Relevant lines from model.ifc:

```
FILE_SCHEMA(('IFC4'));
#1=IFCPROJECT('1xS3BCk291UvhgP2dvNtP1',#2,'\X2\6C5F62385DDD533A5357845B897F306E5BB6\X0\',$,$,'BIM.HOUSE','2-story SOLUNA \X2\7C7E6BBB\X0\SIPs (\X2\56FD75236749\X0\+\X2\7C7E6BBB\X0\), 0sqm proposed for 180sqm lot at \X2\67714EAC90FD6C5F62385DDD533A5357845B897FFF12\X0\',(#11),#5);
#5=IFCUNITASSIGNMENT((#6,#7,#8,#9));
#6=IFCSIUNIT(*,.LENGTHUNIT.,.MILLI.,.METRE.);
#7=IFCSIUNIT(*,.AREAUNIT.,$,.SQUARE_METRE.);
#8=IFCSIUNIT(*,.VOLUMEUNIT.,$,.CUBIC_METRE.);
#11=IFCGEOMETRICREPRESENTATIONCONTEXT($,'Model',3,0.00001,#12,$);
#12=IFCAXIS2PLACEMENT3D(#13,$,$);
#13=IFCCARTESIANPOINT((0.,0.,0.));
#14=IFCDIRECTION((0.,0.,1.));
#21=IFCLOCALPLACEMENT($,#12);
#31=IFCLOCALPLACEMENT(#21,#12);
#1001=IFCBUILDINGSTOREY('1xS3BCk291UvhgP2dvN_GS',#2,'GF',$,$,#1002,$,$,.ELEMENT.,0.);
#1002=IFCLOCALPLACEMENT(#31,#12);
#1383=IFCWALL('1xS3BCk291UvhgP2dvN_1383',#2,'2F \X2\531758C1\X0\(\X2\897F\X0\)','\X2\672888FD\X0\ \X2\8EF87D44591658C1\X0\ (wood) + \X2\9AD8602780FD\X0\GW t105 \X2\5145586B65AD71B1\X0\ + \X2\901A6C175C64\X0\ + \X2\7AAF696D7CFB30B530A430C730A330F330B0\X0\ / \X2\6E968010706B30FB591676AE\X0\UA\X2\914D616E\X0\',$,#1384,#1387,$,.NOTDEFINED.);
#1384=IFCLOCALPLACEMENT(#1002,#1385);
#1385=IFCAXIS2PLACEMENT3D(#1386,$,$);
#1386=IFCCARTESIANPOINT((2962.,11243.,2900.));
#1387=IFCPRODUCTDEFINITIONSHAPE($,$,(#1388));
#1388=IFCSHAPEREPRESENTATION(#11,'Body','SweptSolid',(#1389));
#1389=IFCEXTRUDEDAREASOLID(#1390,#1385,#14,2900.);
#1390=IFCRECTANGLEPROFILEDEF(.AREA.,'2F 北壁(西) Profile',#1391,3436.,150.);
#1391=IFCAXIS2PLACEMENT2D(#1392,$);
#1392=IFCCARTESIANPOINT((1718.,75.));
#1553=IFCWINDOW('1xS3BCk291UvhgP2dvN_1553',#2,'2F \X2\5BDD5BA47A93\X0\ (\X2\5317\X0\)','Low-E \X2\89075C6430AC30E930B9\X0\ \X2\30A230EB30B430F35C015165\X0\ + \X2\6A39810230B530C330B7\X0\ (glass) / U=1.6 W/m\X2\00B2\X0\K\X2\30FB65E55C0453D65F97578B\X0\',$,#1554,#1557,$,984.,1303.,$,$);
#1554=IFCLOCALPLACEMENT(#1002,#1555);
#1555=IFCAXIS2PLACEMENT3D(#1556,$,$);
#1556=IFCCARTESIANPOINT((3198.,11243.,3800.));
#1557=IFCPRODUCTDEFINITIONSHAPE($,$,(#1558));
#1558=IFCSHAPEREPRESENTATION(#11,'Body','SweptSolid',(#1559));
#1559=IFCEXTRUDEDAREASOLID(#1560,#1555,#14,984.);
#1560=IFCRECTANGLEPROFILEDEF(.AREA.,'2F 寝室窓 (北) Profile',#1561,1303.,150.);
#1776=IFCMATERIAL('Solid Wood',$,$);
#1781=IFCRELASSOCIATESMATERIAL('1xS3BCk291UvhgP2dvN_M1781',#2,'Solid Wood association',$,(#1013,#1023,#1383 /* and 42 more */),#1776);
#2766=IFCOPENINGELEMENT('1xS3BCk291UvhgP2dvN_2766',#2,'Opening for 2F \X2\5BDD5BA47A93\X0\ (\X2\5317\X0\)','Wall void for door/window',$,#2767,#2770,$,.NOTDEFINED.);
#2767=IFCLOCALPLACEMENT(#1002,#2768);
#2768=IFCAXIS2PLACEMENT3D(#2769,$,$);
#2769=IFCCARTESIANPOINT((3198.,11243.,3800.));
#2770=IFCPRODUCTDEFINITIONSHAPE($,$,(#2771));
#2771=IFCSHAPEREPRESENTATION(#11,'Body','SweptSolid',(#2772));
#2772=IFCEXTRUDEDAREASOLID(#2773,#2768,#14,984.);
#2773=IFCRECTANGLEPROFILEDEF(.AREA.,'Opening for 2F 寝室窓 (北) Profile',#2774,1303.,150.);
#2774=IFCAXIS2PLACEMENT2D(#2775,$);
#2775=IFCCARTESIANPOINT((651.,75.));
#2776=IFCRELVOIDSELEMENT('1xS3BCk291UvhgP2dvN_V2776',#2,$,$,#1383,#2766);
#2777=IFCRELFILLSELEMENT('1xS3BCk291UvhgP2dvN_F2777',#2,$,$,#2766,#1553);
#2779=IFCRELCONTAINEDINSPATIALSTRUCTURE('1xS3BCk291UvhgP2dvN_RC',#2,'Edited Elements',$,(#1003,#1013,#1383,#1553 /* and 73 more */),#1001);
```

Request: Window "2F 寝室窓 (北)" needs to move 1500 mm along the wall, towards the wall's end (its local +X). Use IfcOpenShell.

```python
import ifcopenshell
import ifcopenshell.api.geometry
import ifcopenshell.util.placement

model = ifcopenshell.open("model.ifc")

window = model.by_guid("1xS3BCk291UvhgP2dvN_1553")
opening = window.FillsVoids[0].RelatingOpeningElement
wall = opening.VoidsElements[0].RelatingBuildingElement

wall_matrix = ifcopenshell.util.placement.get_local_placement(wall.ObjectPlacement)
shift = wall_matrix[:3, 0] * 1500.0
before = ifcopenshell.util.placement.get_local_placement(window.ObjectPlacement)[:3, 3].copy()

# The window is not placed relative to its opening, so move both.
for product in (opening, window):
    matrix = ifcopenshell.util.placement.get_local_placement(product.ObjectPlacement)
    matrix[:3, 3] += shift
    ifcopenshell.api.geometry.edit_object_placement(model, product=product, matrix=matrix, is_si=False)

after = ifcopenshell.util.placement.get_local_placement(window.ObjectPlacement)[:3, 3]
print("window moved by", (after - before).round(3) + 0.0)

model.write("model_rev.ifc")
```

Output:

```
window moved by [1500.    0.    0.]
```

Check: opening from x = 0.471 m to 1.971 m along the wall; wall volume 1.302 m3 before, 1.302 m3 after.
